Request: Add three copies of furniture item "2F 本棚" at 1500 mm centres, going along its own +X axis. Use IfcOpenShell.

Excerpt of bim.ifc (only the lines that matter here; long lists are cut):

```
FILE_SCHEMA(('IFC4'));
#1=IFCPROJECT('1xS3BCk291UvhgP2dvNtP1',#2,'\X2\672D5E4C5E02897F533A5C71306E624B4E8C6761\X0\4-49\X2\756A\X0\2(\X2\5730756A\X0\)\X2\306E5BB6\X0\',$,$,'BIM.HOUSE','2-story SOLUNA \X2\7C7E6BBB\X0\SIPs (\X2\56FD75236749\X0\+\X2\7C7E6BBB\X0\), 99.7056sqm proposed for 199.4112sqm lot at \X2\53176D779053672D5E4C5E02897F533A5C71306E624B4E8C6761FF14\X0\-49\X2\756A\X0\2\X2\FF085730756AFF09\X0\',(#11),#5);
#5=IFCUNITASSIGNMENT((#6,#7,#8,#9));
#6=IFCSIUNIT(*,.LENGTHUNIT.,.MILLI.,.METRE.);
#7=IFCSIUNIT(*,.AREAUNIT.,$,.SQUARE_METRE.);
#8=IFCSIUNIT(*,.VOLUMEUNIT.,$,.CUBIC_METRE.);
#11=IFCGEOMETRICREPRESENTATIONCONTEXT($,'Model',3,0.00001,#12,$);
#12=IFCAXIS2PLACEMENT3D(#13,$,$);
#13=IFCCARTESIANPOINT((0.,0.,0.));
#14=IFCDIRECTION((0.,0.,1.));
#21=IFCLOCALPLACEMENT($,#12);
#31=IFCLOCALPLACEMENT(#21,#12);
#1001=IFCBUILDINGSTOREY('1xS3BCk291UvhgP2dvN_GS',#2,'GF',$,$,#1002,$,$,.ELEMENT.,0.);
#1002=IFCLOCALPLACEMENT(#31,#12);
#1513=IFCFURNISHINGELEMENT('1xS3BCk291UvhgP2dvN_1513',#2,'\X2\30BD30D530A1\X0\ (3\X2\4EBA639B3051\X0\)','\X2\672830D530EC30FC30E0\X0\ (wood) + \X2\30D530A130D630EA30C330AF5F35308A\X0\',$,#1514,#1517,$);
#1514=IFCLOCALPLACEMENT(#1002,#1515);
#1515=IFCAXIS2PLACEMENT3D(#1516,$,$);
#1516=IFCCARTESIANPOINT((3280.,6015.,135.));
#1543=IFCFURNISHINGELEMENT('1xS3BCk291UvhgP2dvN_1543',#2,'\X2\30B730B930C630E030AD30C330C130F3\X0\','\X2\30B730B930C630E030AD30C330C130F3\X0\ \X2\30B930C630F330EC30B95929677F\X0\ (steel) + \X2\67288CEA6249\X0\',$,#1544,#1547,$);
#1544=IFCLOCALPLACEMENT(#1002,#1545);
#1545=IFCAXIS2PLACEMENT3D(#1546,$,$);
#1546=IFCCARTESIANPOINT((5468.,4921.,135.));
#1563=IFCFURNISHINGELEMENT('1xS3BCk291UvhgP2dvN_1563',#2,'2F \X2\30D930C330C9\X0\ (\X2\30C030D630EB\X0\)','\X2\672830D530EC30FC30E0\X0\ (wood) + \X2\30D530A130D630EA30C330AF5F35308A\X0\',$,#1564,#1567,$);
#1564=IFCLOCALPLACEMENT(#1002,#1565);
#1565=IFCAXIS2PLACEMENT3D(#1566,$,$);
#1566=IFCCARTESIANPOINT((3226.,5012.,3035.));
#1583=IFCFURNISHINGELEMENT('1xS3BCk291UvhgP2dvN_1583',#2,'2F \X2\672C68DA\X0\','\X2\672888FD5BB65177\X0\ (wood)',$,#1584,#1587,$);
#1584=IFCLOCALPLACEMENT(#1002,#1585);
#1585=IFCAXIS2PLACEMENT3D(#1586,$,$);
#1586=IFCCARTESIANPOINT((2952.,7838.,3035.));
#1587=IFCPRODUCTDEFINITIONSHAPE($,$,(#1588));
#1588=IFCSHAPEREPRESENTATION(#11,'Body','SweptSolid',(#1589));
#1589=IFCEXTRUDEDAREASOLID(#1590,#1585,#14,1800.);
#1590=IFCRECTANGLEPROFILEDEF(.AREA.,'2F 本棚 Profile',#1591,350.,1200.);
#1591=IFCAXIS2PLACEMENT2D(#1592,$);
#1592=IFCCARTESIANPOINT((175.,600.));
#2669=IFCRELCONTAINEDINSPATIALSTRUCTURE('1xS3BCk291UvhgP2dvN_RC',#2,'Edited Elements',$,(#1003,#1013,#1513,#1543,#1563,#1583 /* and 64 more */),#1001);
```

```python
import ifcopenshell
import ifcopenshell.api.geometry
import ifcopenshell.api.root
import ifcopenshell.util.element
import ifcopenshell.util.placement
import ifcopenshell.util.unit

model = ifcopenshell.open("bim.ifc")
unit_scale = ifcopenshell.util.unit.calculate_unit_scale(model)


def reuse_history(source, copy):
    """copy_class also copies each property set's owner history, people and application; keep the originals."""
    for rel in copy.IsDefinedBy:
        if rel.is_a("IfcRelDefinesByProperties") and (history := rel.RelatingPropertyDefinition.OwnerHistory):
            rel.RelatingPropertyDefinition.OwnerHistory = source.OwnerHistory
            ifcopenshell.util.element.remove_deep2(model, history)


source = model.by_id(1583)
base = ifcopenshell.util.placement.get_local_placement(source.ObjectPlacement)
step = base[:3, 0] * 1.5 / unit_scale

for i in range(1, 4):
    copy = ifcopenshell.api.root.copy_class(model, product=source)
    copy.Representation = ifcopenshell.util.element.copy_deep(
        model, source.Representation, exclude=["IfcGeometricRepresentationContext", "IfcRepresentationMap"]
    )
    reuse_history(source, copy)
    matrix = base.copy()
    matrix[:3, 3] += i * step
    print("added at", matrix[:3, 3].round(3) + 0.0)
    ifcopenshell.api.geometry.edit_object_placement(model, product=copy, matrix=matrix, is_si=False)

model.write("bim_updated.ifc")
```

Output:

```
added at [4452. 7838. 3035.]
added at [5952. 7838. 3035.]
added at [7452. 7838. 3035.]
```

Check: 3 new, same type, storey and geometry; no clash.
